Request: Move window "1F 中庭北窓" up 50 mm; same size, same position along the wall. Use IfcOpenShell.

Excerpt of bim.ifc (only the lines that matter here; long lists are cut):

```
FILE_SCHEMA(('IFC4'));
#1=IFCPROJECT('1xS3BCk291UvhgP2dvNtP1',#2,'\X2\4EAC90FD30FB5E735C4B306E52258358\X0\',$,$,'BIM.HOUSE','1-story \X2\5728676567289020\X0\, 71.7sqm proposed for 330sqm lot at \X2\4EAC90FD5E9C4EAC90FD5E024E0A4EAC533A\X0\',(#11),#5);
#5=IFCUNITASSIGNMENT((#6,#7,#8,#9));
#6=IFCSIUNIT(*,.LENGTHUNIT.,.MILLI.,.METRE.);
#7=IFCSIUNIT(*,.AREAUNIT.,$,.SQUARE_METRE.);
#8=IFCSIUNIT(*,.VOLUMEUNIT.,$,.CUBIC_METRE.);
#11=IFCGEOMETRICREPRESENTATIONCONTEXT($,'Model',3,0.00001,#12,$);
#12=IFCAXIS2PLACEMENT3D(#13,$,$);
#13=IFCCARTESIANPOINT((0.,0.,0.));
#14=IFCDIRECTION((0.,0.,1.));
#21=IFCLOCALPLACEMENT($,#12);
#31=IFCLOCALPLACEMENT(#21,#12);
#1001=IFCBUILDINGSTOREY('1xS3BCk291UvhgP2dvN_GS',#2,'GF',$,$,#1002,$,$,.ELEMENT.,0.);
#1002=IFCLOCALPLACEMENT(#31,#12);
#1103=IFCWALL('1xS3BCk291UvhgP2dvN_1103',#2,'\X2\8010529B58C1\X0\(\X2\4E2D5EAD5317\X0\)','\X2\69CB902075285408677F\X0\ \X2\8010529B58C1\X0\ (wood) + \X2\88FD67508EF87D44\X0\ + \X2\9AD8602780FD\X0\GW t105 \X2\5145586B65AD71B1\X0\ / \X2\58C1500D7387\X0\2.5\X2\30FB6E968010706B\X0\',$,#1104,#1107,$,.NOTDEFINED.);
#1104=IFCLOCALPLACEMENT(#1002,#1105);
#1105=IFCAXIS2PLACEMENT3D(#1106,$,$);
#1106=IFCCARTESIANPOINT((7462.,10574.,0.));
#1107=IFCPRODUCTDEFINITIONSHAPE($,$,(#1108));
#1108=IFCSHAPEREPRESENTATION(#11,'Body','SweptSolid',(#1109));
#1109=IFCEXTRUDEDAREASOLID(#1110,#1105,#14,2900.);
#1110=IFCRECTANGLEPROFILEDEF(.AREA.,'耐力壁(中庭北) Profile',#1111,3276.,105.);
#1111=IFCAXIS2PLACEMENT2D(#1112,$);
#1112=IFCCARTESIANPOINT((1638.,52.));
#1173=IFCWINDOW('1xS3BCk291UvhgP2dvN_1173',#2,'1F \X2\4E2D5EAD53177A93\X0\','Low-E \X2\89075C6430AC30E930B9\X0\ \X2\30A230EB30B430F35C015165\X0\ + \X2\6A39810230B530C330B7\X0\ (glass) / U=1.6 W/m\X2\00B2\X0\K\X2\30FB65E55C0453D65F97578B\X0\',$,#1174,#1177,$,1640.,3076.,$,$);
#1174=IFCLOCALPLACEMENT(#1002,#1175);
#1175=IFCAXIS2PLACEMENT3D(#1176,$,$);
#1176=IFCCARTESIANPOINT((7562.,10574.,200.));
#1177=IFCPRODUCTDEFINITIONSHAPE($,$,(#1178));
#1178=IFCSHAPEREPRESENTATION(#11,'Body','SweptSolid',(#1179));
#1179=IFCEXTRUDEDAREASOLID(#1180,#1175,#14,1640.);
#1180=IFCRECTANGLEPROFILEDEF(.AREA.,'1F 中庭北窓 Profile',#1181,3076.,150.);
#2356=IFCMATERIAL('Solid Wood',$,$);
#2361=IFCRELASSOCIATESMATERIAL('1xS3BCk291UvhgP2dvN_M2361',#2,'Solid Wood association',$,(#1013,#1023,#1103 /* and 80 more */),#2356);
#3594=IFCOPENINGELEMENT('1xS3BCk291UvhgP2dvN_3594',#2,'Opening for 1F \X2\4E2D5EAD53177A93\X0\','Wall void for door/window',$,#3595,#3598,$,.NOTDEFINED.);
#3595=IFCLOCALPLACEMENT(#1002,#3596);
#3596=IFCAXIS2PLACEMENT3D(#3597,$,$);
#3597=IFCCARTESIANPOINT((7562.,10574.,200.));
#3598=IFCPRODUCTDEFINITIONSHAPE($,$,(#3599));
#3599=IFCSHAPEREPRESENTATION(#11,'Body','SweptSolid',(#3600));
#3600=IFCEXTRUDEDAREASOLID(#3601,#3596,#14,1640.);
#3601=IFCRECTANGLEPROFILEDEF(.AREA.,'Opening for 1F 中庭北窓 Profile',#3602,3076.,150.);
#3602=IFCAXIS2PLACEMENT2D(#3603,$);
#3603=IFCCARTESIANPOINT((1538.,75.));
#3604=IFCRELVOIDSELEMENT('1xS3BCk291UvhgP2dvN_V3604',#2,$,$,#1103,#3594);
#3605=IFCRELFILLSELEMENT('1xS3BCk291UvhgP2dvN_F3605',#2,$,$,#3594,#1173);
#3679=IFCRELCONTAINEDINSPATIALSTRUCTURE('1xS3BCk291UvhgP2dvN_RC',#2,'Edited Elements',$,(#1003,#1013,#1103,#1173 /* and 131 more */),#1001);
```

```python
import numpy as np
import ifcopenshell
import ifcopenshell.api.geometry
import ifcopenshell.util.placement
import ifcopenshell.util.unit

model = ifcopenshell.open("bim.ifc")
unit_scale = ifcopenshell.util.unit.calculate_unit_scale(model)

window = model.by_guid("1xS3BCk291UvhgP2dvN_1173")
opening = window.FillsVoids[0].RelatingOpeningElement
dz = 0.05 / unit_scale

shift = np.array([0.0, 0.0, dz])
# The window is not placed relative to its opening, so move both.
for product in (opening, window):
    matrix = ifcopenshell.util.placement.get_local_placement(product.ObjectPlacement)
    matrix[:3, 3] += shift
    ifcopenshell.api.geometry.edit_object_placement(model, product=product, matrix=matrix, is_si=False)

print(f"moved by {dz * unit_scale:+.3f} m")

model.write("bim_edited.ifc")
```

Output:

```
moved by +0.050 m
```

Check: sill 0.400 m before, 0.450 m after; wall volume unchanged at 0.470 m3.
